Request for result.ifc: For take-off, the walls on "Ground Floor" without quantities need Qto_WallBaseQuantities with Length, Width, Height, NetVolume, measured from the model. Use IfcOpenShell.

First a look at what the model holds.

```python
import ifcopenshell
import ifcopenshell.util.element
import ifcopenshell.util.unit

model = ifcopenshell.open("result.ifc")
print(model.schema)
for unit_type in ("LENGTHUNIT", "AREAUNIT", "VOLUMEUNIT"):
    print(unit_type, ifcopenshell.util.unit.calculate_unit_scale(model, unit_type))
storey = next(s for s in model.by_type("IfcBuildingStorey") if s.Name == "Ground Floor")
walls = [e for e in ifcopenshell.util.element.get_decomposition(storey) if e.is_a("IfcWall")]
for e in sorted(walls, key=lambda e: e.id()):
    print(e.id(), e.is_a(), e.Name, list(ifcopenshell.util.element.get_psets(e, qtos_only=True)), sep=" | ")
```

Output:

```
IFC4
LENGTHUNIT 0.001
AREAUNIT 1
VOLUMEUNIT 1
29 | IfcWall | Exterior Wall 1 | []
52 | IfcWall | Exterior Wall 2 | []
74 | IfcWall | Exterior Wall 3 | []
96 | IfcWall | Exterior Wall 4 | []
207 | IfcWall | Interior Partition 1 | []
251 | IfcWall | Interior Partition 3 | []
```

```python
import ifcopenshell
import ifcopenshell.api.pset
import ifcopenshell.geom
import ifcopenshell.util.element
import ifcopenshell.util.shape
import ifcopenshell.util.unit

model = ifcopenshell.open("result.ifc")
unit_scale = ifcopenshell.util.unit.calculate_unit_scale(model)
volume_scale = ifcopenshell.util.unit.calculate_unit_scale(model, "VOLUMEUNIT")
settings = ifcopenshell.geom.settings()

storey = next(s for s in model.by_type("IfcBuildingStorey") if s.Name == "Ground Floor")
walls = [e for e in ifcopenshell.util.element.get_decomposition(storey) if e.is_a("IfcWall")]

for e in sorted(walls, key=lambda e: e.id()):
    if ifcopenshell.util.element.get_psets(e, qtos_only=True, should_inherit=False):
        continue
    # Geometry comes back in metres, in the element's own axes.
    shape = ifcopenshell.geom.create_shape(settings, e)
    values = {
        "Length": ifcopenshell.util.shape.get_x(shape.geometry) / unit_scale,
        "Width": ifcopenshell.util.shape.get_y(shape.geometry) / unit_scale,
        "Height": ifcopenshell.util.shape.get_z(shape.geometry) / unit_scale,
        "NetVolume": ifcopenshell.util.shape.get_volume(shape.geometry) / volume_scale,
    }
    qto = ifcopenshell.api.pset.add_qto(model, product=e, name="Qto_WallBaseQuantities")
    ifcopenshell.api.pset.edit_qto(model, qto=qto, properties=values)
    print(e.id(), {k: round(v, 3) for k, v in values.items()})

model.write("result-out.ifc")
```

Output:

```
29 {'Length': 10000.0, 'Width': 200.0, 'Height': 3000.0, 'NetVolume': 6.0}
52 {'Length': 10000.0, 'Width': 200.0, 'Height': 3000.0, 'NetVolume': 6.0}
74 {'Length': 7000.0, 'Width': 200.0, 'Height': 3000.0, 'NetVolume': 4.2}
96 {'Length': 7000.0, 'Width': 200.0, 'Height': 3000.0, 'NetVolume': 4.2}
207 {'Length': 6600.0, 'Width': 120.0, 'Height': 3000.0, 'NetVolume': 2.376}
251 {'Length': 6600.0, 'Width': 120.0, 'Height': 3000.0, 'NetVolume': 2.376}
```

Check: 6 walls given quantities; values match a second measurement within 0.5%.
